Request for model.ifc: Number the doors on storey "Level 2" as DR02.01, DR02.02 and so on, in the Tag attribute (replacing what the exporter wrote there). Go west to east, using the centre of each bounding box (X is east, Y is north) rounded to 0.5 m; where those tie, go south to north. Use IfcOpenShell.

First a look at what the model holds.

```python
import ifcopenshell
import ifcopenshell.util.element
import ifcopenshell.util.placement

model = ifcopenshell.open("model.ifc")
print(model.schema)
storey = next(s for s in model.by_type("IfcBuildingStorey") if s.Name == "Level 2")
doors = [e for e in ifcopenshell.util.element.get_decomposition(storey) if e.is_a("IfcDoor")]
for e in sorted(doors, key=lambda e: e.id()):
    origin = ifcopenshell.util.placement.get_local_placement(e.ObjectPlacement)[:3, 3]
    print(e.id(), e.Tag, e.Name, origin.round(2) + 0.0, sep=" | ")
```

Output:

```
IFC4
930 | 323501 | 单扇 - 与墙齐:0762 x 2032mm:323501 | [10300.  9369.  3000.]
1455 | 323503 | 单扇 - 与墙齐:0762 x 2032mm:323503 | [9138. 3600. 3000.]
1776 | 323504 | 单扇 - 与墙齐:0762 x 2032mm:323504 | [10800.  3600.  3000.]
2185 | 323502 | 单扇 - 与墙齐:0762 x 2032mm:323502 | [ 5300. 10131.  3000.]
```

```python
import ifcopenshell
import ifcopenshell.geom
import ifcopenshell.util.element
import ifcopenshell.util.shape

model = ifcopenshell.open("model.ifc")
settings = ifcopenshell.geom.settings()
settings.set("use-world-coords", True)


def centre(element):
    shape = ifcopenshell.geom.create_shape(settings, element)
    return ifcopenshell.util.shape.get_bbox_centroid(shape.geometry)


storey = next(s for s in model.by_type("IfcBuildingStorey") if s.Name == "Level 2")
doors = [e for e in ifcopenshell.util.element.get_decomposition(storey) if e.is_a("IfcDoor")]

# Insertion points can sit at a corner or the storey origin, so sort by the geometry (in metres).
centres = {e: centre(e) for e in doors}
doors.sort(key=lambda e: (round(centres[e][0] / 0.5), centres[e][1]))

for i, e in enumerate(doors, start=1):
    number = f"DR02.{i:02d}"
    e.Tag = number
    print(e.id(), number)

model.write("model_updated.ifc")
```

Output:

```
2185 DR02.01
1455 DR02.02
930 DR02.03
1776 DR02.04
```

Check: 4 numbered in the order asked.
